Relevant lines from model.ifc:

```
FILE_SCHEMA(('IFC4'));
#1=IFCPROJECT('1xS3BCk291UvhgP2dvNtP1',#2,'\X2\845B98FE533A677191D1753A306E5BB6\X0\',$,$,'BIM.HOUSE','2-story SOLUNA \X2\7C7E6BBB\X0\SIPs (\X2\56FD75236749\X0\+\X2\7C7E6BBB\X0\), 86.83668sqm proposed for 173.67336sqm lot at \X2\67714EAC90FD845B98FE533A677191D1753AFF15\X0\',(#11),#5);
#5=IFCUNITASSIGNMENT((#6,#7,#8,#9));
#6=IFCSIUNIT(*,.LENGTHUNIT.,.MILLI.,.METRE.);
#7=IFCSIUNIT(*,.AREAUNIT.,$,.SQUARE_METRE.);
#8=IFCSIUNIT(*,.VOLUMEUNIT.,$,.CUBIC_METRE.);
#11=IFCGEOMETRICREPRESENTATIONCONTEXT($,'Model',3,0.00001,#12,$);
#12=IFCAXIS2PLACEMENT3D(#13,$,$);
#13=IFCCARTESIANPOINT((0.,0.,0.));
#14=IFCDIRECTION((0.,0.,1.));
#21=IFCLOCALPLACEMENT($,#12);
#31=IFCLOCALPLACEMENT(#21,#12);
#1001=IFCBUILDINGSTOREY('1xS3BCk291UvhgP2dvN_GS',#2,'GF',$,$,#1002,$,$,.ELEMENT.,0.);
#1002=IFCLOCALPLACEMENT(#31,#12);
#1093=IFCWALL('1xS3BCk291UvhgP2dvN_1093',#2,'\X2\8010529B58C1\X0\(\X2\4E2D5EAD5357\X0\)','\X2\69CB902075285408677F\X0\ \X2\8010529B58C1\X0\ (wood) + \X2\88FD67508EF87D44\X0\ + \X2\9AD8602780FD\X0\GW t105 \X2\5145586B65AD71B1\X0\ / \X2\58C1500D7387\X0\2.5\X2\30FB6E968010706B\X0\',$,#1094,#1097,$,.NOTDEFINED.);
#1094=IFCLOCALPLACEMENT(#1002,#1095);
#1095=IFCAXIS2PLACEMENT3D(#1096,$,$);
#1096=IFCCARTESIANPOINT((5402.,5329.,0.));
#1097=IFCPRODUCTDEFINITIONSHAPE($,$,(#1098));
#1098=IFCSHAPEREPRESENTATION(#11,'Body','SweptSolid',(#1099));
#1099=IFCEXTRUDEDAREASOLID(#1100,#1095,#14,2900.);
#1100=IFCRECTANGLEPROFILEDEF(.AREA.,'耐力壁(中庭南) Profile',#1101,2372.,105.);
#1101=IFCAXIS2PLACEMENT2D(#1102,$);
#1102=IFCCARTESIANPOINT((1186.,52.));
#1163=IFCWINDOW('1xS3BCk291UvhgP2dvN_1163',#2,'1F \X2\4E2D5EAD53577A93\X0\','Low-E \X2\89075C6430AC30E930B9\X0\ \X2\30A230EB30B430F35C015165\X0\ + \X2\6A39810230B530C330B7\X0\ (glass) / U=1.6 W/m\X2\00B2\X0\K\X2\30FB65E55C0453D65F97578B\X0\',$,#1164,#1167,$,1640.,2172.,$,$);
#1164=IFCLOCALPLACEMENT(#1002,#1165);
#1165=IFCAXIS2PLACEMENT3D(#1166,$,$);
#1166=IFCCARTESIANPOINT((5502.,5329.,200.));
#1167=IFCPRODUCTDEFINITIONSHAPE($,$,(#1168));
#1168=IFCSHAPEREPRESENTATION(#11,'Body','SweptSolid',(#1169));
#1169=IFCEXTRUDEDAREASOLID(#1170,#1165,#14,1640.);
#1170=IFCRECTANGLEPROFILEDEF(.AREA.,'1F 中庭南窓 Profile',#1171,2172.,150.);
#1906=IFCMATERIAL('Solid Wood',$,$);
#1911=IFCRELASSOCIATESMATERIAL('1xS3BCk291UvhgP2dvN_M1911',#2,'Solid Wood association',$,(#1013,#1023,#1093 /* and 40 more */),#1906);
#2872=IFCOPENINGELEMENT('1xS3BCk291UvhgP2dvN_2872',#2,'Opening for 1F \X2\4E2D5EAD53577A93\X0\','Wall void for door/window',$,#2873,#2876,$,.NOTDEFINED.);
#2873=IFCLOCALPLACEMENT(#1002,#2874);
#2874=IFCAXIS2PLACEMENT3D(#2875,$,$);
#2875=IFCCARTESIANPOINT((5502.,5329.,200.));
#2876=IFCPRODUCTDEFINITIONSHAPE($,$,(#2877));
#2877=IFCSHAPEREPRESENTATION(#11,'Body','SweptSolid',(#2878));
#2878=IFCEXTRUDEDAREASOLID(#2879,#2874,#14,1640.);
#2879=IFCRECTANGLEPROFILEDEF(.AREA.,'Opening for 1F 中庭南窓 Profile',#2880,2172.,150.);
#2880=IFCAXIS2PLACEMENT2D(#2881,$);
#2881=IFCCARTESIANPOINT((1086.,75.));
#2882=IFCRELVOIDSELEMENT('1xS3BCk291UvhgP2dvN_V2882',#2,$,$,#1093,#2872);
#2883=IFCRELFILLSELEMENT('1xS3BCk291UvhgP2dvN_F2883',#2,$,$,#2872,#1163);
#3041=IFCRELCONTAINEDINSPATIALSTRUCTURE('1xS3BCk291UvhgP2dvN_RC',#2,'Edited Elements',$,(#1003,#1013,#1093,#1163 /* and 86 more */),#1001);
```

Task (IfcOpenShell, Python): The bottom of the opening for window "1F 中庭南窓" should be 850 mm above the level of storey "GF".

```python
import numpy as np
import ifcopenshell
import ifcopenshell.api.geometry
import ifcopenshell.geom
import ifcopenshell.util.element
import ifcopenshell.util.placement
import ifcopenshell.util.shape
import ifcopenshell.util.unit

model = ifcopenshell.open("model.ifc")
unit_scale = ifcopenshell.util.unit.calculate_unit_scale(model)

window = model.by_id(1163)
opening = window.FillsVoids[0].RelatingOpeningElement
storey = ifcopenshell.util.element.get_container(window, ifc_class="IfcBuildingStorey")
level = ifcopenshell.util.placement.get_local_placement(storey.ObjectPlacement)[2, 3]

# The opening's origin need not be at the sill, so measure its lowest point.
shape = ifcopenshell.geom.create_shape(ifcopenshell.geom.settings(), opening)
bottom = ifcopenshell.util.shape.get_shape_bottom_elevation(shape, shape.geometry) / unit_scale
dz = level + 0.85 / unit_scale - bottom

shift = np.array([0.0, 0.0, dz])
# The window is not placed relative to its opening, so move both.
for product in (opening, window):
    matrix = ifcopenshell.util.placement.get_local_placement(product.ObjectPlacement)
    matrix[:3, 3] += shift
    ifcopenshell.api.geometry.edit_object_placement(model, product=product, matrix=matrix, is_si=False)

print(f"moved by {dz * unit_scale:+.3f} m")

model.write("model_edited.ifc")
```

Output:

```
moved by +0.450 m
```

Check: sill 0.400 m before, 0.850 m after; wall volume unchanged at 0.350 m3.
